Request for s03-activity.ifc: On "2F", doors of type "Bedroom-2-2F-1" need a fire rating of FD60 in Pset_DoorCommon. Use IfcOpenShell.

First a look at what the model holds.

```python
import ifcopenshell
import ifcopenshell.util.element

model = ifcopenshell.open("s03-activity.ifc")
print(model.schema)
storey = next(s for s in model.by_type("IfcBuildingStorey") if s.Name == "2F")
doors = [e for e in ifcopenshell.util.element.get_decomposition(storey) if e.is_a("IfcDoor")]
seen = {}
for e in doors:
    element_type = ifcopenshell.util.element.get_type(e)
    key = (element_type.Name if element_type != e and element_type else None, ifcopenshell.util.element.get_pset(e, "Pset_DoorCommon", "FireRating"))
    seen[key] = seen.get(key, 0) + 1
for (name, value), count in sorted(seen.items(), key=str):
    print(count, "x", name, "|", value)
```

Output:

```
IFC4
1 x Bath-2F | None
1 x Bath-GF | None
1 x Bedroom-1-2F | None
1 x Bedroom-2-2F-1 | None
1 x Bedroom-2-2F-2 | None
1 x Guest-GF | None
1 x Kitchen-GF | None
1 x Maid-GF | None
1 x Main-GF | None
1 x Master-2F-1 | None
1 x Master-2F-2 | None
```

```python
import ifcopenshell
import ifcopenshell.api.pset
import ifcopenshell.util.element

model = ifcopenshell.open("s03-activity.ifc")

storey = next(s for s in model.by_type("IfcBuildingStorey") if s.Name == "2F")
doors = [e for e in ifcopenshell.util.element.get_decomposition(storey) if e.is_a("IfcDoor")]

count = 0
for e in doors:
    element_type = ifcopenshell.util.element.get_type(e)
    if element_type in (None, e) or element_type.Name != "Bedroom-2-2F-1":
        continue
    # add_pset returns the element's existing set when there is one.
    pset = ifcopenshell.api.pset.add_pset(model, product=e, name="Pset_DoorCommon")
    ifcopenshell.api.pset.edit_pset(model, pset=pset, properties={"FireRating": "FD60"})
    count += 1

print(count, "doors updated")

model.write("s03-activity_updated.ifc")
```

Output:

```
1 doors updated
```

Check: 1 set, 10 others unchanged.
